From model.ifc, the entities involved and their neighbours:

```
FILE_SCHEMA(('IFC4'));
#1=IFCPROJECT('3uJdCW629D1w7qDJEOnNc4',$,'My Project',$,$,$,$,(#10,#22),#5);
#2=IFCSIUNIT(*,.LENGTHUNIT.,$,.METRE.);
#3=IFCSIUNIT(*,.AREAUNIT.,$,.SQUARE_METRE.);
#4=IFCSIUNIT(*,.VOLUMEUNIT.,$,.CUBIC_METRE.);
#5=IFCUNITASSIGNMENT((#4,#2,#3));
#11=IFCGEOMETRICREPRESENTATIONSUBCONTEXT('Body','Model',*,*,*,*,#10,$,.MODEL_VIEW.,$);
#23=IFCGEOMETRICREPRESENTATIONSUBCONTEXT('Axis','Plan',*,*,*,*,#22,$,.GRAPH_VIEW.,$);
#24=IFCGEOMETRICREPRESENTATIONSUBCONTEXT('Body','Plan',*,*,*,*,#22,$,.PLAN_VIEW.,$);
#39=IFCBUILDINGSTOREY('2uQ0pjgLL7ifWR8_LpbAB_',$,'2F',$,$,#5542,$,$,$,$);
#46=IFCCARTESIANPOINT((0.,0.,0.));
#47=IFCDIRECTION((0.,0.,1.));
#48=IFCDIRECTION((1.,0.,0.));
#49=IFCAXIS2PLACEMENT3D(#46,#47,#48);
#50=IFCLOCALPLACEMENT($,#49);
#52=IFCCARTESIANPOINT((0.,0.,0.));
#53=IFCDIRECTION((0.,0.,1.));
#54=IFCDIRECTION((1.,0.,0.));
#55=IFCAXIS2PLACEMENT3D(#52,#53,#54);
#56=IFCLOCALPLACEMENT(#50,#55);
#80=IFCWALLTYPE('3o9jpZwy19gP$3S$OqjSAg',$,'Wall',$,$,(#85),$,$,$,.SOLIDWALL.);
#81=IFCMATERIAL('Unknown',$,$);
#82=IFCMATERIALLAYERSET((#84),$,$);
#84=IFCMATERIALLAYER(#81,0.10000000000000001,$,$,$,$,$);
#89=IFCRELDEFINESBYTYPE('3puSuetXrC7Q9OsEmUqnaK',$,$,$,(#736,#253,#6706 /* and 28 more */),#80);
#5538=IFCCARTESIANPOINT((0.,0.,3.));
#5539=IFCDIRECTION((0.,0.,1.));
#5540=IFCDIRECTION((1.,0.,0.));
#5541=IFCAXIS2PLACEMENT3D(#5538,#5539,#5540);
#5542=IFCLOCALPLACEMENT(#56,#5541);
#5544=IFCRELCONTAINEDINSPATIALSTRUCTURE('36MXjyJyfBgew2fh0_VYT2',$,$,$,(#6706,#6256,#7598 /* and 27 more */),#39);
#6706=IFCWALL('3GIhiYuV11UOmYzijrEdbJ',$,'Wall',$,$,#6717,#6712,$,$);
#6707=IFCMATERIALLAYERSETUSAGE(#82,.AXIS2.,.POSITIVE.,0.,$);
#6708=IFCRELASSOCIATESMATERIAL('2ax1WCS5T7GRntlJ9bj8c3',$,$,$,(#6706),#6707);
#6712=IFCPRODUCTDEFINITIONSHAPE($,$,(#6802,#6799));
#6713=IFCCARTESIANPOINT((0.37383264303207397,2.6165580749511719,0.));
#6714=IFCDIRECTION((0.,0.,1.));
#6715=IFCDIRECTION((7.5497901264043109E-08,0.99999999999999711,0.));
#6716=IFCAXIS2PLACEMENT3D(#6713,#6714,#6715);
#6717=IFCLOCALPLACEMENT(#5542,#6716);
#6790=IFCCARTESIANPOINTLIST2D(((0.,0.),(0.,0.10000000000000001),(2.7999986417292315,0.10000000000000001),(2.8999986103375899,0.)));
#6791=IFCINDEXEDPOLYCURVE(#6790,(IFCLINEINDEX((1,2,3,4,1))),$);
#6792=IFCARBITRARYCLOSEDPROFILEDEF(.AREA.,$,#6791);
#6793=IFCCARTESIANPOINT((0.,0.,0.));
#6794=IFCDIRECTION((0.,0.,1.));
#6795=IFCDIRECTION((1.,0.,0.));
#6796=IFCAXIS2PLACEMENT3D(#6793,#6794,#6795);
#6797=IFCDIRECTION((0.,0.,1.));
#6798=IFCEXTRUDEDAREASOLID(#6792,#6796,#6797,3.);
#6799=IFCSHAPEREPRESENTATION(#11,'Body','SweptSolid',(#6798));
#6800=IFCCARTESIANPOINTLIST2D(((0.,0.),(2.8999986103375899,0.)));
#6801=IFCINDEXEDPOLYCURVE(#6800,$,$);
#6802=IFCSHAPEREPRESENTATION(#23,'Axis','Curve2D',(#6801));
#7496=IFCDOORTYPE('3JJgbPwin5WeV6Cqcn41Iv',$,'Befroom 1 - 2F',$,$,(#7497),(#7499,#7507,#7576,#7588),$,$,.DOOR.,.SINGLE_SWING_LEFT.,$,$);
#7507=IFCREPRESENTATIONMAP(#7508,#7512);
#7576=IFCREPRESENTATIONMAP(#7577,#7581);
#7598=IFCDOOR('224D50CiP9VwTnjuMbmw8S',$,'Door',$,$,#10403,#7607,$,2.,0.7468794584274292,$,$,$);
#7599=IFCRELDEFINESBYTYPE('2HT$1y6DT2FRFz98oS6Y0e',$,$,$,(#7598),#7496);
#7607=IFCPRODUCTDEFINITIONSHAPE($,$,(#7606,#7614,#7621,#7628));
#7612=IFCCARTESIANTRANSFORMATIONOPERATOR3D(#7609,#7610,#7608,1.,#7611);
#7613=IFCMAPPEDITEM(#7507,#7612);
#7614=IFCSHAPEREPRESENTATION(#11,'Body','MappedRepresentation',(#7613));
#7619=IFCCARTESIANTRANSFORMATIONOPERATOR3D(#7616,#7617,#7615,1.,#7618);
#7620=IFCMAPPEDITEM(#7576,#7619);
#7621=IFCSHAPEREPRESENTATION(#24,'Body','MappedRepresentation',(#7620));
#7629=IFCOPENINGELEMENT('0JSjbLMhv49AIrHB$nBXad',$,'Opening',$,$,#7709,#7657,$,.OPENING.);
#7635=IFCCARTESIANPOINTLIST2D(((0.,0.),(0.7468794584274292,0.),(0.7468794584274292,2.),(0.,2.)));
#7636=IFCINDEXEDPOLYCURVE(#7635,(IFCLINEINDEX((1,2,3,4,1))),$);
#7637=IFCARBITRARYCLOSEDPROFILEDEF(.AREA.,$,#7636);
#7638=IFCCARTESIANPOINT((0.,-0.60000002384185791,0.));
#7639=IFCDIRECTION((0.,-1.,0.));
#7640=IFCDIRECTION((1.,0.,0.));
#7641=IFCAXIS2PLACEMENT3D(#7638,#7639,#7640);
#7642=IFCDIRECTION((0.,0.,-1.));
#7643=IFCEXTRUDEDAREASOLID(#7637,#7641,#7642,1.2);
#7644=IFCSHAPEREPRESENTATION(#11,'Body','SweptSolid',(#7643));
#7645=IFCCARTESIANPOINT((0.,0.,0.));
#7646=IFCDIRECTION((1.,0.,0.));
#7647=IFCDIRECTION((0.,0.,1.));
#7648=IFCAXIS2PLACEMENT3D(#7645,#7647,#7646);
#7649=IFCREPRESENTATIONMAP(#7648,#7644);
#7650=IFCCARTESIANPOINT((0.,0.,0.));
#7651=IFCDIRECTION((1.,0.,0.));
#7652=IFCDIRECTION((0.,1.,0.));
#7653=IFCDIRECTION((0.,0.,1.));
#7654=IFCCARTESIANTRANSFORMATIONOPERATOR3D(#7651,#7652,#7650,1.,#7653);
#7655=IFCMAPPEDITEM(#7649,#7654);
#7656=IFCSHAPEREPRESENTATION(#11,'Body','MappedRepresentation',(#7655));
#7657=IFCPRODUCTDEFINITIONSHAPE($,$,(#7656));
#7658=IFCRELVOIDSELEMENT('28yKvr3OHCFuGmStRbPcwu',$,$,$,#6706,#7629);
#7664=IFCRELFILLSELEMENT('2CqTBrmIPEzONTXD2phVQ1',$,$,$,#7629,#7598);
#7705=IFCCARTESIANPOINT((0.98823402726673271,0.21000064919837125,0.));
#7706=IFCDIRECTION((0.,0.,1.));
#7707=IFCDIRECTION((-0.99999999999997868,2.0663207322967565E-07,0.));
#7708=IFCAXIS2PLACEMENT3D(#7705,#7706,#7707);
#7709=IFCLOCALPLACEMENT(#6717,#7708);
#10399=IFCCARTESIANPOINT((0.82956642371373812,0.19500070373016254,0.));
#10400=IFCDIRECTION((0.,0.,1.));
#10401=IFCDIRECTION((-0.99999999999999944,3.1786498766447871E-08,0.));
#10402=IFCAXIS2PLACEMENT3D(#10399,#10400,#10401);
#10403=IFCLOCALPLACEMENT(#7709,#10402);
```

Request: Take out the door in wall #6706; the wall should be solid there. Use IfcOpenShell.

```python
import ifcopenshell
import ifcopenshell.api.feature
import ifcopenshell.api.root
import ifcopenshell.geom
import ifcopenshell.util.shape

model = ifcopenshell.open("model.ifc")
settings = ifcopenshell.geom.settings()


def volume(element):
    """Net volume in cubic metres, openings subtracted."""
    shape = ifcopenshell.geom.create_shape(settings, element)
    return ifcopenshell.util.shape.get_volume(shape.geometry)


door = model.by_guid("224D50CiP9VwTnjuMbmw8S")
opening = door.FillsVoids[0].RelatingOpeningElement
wall = opening.VoidsElements[0].RelatingBuildingElement
before = volume(wall)

ifcopenshell.api.root.remove_product(model, product=door)
ifcopenshell.api.feature.remove_feature(model, feature=opening)

after = volume(wall)

print(f"wall volume {before:.3f} -> {after:.3f} m3")

model.write("model_rev.ifc")
```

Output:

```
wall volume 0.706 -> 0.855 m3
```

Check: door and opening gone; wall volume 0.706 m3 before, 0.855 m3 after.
